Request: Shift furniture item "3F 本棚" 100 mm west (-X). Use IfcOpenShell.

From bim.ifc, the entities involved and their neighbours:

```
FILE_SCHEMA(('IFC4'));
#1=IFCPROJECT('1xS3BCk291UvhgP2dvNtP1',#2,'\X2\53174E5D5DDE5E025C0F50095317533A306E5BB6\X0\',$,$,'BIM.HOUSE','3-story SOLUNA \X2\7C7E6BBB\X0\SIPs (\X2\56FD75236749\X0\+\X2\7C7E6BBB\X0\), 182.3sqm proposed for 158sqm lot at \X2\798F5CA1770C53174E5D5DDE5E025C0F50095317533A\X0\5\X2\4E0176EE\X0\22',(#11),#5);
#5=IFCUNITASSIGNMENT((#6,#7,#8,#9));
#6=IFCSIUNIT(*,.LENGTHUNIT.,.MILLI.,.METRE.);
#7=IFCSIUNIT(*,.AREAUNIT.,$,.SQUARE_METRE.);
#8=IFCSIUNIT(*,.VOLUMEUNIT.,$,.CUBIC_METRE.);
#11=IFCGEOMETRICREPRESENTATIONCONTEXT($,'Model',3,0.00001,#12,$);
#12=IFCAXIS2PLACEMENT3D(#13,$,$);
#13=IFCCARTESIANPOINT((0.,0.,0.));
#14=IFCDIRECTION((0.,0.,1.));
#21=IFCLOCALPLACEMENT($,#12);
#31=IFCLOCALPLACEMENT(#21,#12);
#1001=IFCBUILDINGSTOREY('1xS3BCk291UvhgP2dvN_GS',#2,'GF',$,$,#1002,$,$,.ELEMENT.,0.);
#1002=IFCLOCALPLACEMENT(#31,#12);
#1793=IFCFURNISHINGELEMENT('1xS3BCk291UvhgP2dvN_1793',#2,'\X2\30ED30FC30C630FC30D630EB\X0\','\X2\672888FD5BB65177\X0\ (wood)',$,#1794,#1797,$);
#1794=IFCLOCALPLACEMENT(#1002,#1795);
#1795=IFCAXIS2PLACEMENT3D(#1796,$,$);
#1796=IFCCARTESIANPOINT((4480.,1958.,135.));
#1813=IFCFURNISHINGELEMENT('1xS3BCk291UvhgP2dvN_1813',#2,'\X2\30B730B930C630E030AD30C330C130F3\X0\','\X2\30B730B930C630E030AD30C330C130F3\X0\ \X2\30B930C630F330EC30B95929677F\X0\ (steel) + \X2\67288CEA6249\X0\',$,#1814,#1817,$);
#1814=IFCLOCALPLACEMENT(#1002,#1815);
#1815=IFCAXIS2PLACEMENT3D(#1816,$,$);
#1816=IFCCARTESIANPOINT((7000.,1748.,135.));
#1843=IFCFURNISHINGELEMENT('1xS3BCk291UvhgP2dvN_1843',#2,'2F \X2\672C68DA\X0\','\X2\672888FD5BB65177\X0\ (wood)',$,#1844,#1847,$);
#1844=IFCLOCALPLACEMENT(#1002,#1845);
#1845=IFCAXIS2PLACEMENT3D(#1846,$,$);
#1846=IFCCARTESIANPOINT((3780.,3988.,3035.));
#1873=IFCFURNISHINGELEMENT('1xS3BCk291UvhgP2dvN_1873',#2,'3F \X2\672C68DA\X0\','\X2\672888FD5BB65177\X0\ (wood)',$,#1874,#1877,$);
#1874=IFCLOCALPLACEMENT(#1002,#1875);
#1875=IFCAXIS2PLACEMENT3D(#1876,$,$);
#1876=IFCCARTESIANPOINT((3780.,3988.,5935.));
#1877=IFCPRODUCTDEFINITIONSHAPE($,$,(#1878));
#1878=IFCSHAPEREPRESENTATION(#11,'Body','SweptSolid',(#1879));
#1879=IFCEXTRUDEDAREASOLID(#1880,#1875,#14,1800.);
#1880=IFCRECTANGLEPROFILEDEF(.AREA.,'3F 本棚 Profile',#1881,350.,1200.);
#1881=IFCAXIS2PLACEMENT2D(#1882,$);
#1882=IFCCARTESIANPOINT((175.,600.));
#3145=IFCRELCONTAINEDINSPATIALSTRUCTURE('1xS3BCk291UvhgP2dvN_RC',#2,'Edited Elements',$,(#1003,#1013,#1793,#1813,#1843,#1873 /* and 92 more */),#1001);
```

```python
import ifcopenshell
import ifcopenshell.api.geometry
import ifcopenshell.util.placement

model = ifcopenshell.open("bim.ifc")

item = model.by_guid("1xS3BCk291UvhgP2dvN_1873")
matrix = ifcopenshell.util.placement.get_local_placement(item.ObjectPlacement)
matrix[0, 3] -= 100.0
ifcopenshell.api.geometry.edit_object_placement(model, product=item, matrix=matrix, is_si=False)

print(ifcopenshell.util.placement.get_local_placement(item.ObjectPlacement).round(3) + 0.0)

model.write("bim_rev.ifc")
```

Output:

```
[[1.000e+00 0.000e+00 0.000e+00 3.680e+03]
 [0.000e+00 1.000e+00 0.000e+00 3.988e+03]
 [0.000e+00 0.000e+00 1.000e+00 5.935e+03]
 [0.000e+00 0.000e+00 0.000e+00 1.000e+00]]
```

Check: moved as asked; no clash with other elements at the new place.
